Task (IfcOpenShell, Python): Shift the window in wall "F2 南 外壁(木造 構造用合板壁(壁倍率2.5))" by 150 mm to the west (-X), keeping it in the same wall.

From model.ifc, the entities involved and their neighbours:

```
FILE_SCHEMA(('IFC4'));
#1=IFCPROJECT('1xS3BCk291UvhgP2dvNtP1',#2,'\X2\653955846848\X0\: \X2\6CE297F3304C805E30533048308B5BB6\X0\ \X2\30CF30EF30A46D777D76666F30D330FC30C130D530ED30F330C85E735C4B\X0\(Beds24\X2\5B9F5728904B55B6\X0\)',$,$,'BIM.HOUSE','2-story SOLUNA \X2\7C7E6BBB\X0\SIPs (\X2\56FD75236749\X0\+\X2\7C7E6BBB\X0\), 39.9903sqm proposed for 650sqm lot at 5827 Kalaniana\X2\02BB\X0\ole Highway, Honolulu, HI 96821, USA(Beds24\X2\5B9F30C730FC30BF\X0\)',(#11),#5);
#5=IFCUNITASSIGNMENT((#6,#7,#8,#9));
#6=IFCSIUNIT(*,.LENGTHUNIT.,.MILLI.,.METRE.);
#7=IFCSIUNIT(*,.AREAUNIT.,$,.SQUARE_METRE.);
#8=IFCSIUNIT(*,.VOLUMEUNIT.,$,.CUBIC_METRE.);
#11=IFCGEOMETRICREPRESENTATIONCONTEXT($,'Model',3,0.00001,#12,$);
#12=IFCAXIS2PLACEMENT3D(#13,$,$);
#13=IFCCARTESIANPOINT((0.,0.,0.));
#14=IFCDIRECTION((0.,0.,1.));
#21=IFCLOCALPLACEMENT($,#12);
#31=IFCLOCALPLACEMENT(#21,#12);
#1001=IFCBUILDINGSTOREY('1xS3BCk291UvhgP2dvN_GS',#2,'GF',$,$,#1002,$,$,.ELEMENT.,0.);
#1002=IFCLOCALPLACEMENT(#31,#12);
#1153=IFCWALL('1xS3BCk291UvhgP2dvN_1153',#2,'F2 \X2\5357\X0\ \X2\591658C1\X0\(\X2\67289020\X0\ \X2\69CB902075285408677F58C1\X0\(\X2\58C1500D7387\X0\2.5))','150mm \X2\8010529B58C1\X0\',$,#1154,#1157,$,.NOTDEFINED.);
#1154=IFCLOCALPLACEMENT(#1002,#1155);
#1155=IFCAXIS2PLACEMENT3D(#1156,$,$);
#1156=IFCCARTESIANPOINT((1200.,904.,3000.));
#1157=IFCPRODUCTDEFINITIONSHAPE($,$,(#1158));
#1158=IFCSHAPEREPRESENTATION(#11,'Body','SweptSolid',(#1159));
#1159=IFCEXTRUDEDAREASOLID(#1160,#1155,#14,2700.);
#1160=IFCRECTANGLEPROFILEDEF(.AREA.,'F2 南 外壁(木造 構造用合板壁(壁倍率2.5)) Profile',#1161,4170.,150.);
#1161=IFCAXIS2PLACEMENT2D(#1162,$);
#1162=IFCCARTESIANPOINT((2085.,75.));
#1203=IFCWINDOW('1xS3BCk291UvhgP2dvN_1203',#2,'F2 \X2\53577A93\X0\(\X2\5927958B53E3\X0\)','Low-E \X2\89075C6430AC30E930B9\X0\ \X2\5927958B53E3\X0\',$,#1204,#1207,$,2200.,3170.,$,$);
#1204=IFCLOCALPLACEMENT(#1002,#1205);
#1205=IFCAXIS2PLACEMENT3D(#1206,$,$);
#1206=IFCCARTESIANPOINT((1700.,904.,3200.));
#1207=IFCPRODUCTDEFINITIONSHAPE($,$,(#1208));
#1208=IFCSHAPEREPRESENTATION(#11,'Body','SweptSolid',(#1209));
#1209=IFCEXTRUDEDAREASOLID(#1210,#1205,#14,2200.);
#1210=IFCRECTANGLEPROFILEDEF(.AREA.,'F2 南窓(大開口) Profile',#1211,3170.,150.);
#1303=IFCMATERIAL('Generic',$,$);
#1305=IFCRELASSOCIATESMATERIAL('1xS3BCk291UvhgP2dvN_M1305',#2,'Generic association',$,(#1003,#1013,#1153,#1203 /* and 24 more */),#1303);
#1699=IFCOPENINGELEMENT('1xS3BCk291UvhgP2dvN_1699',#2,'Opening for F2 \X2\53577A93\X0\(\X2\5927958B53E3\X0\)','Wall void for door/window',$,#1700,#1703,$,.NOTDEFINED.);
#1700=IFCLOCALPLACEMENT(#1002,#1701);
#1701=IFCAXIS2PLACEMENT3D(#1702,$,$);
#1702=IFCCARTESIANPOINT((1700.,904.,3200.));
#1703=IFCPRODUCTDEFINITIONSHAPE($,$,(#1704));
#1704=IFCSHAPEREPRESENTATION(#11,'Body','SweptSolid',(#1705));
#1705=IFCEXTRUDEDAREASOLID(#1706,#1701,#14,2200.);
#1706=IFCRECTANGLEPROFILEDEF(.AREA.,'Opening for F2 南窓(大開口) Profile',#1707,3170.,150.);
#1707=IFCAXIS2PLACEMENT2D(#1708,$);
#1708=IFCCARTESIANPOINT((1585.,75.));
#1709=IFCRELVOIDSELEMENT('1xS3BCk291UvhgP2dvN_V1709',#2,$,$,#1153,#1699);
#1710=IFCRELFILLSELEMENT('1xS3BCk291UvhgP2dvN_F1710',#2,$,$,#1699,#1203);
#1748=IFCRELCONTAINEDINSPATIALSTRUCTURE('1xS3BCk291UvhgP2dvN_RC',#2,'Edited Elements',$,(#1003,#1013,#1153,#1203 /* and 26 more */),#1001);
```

```python
import ifcopenshell
import ifcopenshell.api.geometry
import ifcopenshell.util.placement
import ifcopenshell.util.unit

model = ifcopenshell.open("model.ifc")
unit_scale = ifcopenshell.util.unit.calculate_unit_scale(model)

window = model.by_id(1203)
opening = window.FillsVoids[0].RelatingOpeningElement
wall = opening.VoidsElements[0].RelatingBuildingElement

wall_matrix = ifcopenshell.util.placement.get_local_placement(wall.ObjectPlacement)
shift = wall_matrix[:3, 0] * -0.15 / unit_scale
before = ifcopenshell.util.placement.get_local_placement(window.ObjectPlacement)[:3, 3].copy()

# The window is not placed relative to its opening, so move both.
for product in (opening, window):
    matrix = ifcopenshell.util.placement.get_local_placement(product.ObjectPlacement)
    matrix[:3, 3] += shift
    ifcopenshell.api.geometry.edit_object_placement(model, product=product, matrix=matrix, is_si=False)

after = ifcopenshell.util.placement.get_local_placement(window.ObjectPlacement)[:3, 3]
print("window moved by", (after - before).round(3) + 0.0)

model.write("model-out.ifc")
```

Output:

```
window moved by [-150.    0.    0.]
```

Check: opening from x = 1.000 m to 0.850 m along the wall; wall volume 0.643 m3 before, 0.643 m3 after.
